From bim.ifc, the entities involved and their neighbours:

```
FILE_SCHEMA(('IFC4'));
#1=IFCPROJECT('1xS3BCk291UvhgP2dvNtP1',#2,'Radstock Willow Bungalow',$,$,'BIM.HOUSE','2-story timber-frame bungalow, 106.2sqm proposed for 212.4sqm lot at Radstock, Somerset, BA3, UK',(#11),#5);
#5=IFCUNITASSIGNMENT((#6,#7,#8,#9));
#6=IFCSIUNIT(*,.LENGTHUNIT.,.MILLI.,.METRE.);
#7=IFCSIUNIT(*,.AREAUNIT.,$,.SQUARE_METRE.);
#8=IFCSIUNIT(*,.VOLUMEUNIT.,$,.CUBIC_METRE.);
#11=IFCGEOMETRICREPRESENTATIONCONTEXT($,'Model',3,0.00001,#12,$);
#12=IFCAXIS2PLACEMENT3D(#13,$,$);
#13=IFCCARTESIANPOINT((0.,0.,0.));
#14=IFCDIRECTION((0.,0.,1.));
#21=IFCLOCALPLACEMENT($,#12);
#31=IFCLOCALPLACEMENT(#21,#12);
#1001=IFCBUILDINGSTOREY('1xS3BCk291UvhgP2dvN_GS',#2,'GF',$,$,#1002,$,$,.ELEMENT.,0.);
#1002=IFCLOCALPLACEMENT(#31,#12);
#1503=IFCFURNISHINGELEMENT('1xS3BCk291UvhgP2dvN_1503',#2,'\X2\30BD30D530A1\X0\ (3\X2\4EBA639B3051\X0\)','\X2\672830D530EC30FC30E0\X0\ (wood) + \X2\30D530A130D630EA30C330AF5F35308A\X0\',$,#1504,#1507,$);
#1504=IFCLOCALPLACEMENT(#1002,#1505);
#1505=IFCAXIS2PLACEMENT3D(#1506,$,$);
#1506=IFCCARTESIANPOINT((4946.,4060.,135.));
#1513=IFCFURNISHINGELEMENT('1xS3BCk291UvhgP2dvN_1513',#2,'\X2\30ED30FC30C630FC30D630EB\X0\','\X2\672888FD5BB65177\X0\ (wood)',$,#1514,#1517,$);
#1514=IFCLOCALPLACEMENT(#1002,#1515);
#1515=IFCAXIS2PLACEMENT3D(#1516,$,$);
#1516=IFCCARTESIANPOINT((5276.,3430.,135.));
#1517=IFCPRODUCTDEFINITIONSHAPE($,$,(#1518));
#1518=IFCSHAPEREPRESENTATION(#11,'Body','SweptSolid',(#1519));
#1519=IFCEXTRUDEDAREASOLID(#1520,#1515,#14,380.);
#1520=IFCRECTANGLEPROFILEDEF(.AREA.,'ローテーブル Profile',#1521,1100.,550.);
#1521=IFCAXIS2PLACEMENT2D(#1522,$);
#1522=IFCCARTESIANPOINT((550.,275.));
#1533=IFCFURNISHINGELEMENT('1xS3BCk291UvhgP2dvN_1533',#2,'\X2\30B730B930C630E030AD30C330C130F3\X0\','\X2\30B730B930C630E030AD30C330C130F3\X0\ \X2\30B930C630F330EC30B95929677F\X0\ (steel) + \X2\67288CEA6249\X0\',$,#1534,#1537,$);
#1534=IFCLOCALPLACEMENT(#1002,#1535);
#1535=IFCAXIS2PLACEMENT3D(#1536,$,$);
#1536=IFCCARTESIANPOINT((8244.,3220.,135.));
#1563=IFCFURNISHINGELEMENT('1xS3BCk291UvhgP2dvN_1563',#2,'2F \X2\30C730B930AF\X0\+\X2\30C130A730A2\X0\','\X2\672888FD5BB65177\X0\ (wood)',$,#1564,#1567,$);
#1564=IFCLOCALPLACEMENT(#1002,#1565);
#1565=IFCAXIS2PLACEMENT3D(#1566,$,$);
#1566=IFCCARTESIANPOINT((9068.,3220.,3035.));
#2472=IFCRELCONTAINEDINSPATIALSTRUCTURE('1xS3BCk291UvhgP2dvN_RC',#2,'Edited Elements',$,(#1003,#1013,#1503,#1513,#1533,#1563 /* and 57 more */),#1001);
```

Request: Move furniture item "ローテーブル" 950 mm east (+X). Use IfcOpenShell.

```python
import ifcopenshell
import ifcopenshell.api.geometry
import ifcopenshell.util.placement
import ifcopenshell.util.unit

model = ifcopenshell.open("bim.ifc")
unit_scale = ifcopenshell.util.unit.calculate_unit_scale(model)

item = model.by_guid("1xS3BCk291UvhgP2dvN_1513")
matrix = ifcopenshell.util.placement.get_local_placement(item.ObjectPlacement)
matrix[0, 3] += 0.95 / unit_scale
ifcopenshell.api.geometry.edit_object_placement(model, product=item, matrix=matrix, is_si=False)

print(ifcopenshell.util.placement.get_local_placement(item.ObjectPlacement).round(3) + 0.0)

model.write("bim_rev.ifc")
```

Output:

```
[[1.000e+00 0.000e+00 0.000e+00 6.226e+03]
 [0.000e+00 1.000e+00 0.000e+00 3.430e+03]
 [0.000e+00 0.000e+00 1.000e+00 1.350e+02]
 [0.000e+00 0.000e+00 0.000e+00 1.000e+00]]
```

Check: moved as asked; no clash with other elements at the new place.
